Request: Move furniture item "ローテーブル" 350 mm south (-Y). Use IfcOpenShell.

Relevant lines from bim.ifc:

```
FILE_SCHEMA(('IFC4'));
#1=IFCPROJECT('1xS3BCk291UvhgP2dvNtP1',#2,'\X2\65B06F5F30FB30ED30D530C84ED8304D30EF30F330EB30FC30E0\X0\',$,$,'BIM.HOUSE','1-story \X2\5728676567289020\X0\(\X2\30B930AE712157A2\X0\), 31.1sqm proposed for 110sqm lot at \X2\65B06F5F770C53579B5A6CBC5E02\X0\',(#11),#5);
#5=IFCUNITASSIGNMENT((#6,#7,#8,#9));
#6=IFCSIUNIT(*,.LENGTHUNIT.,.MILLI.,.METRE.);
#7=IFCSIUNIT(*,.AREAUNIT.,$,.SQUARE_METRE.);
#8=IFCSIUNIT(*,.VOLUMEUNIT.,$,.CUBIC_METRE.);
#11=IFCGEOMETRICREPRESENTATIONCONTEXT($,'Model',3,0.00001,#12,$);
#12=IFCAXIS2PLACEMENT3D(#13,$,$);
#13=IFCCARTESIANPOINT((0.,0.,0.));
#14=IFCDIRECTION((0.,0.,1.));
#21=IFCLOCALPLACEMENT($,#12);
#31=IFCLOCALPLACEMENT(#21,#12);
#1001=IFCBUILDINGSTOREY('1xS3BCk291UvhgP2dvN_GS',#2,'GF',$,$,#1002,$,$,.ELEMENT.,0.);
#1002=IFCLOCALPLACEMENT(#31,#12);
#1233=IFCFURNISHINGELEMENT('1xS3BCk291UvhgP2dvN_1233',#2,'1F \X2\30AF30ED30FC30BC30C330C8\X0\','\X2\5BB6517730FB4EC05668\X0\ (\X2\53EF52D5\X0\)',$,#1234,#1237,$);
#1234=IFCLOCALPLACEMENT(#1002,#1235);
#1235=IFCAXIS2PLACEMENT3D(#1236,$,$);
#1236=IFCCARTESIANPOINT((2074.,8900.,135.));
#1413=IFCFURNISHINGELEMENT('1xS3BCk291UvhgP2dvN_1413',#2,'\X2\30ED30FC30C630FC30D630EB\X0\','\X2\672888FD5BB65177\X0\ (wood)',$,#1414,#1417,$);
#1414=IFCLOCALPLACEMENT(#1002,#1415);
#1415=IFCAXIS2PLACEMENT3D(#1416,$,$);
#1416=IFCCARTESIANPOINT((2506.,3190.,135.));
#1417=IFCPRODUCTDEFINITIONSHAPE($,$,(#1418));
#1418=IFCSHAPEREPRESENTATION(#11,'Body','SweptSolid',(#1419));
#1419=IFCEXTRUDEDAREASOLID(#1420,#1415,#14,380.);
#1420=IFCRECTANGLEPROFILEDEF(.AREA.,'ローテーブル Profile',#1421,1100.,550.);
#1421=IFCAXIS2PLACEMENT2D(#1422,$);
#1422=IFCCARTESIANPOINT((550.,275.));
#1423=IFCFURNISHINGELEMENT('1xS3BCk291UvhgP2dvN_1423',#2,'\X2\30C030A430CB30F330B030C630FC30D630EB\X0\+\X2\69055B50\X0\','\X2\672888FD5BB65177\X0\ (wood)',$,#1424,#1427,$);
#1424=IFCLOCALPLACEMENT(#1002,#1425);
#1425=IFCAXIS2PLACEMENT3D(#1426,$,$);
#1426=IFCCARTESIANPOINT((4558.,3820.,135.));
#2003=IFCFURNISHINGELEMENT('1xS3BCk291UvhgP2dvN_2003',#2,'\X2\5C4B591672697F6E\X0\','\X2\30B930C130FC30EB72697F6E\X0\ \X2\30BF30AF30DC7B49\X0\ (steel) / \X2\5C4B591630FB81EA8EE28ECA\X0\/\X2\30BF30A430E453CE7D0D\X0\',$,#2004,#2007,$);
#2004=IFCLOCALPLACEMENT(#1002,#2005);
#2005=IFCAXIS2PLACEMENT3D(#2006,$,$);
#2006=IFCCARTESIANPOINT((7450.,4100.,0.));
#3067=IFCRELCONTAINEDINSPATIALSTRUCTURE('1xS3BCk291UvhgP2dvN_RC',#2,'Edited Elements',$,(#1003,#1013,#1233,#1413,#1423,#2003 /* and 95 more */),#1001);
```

```python
import ifcopenshell
import ifcopenshell.api.geometry
import ifcopenshell.util.placement
import ifcopenshell.util.unit

model = ifcopenshell.open("bim.ifc")
unit_scale = ifcopenshell.util.unit.calculate_unit_scale(model)

item = model.by_guid("1xS3BCk291UvhgP2dvN_1413")
matrix = ifcopenshell.util.placement.get_local_placement(item.ObjectPlacement)
matrix[1, 3] -= 0.35 / unit_scale
ifcopenshell.api.geometry.edit_object_placement(model, product=item, matrix=matrix, is_si=False)

print(ifcopenshell.util.placement.get_local_placement(item.ObjectPlacement).round(3) + 0.0)

model.write("bim_edited.ifc")
```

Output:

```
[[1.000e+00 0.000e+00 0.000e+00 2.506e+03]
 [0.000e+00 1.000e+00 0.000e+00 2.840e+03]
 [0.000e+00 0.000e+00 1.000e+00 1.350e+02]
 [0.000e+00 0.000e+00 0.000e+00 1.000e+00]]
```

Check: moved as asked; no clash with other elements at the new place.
